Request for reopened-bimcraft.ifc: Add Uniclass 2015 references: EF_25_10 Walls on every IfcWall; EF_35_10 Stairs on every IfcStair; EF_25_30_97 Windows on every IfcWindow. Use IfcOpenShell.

First a look at what the model holds.

```python
import ifcopenshell

model = ifcopenshell.open("reopened-bimcraft.ifc")
print(model.schema)
print("classifications:", [c.Name for c in model.by_type("IfcClassification")])
for ifc_class in ("IfcDoor", "IfcRoof", "IfcStair", "IfcWall", "IfcWindow"):
    print(ifc_class, len(model.by_type(ifc_class)))
```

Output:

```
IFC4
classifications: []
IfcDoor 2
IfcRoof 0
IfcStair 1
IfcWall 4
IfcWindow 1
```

```python
import ifcopenshell
import ifcopenshell.api.classification

model = ifcopenshell.open("reopened-bimcraft.ifc")

system = ifcopenshell.api.classification.add_classification(model, classification="Uniclass 2015")

codes = {
    "IfcWall": ("EF_25_10", "Walls"),
    "IfcStair": ("EF_35_10", "Stairs"),
    "IfcWindow": ("EF_25_30_97", "Windows"),
}
for ifc_class, (code, name) in codes.items():
    products = model.by_type(ifc_class)
    ifcopenshell.api.classification.add_reference(
        model, products=products, classification=system, identification=code, name=name
    )
    print(code, len(products))

model.write("reopened-bimcraft_updated.ifc")
```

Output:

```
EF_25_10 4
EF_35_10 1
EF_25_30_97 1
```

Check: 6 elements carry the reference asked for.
